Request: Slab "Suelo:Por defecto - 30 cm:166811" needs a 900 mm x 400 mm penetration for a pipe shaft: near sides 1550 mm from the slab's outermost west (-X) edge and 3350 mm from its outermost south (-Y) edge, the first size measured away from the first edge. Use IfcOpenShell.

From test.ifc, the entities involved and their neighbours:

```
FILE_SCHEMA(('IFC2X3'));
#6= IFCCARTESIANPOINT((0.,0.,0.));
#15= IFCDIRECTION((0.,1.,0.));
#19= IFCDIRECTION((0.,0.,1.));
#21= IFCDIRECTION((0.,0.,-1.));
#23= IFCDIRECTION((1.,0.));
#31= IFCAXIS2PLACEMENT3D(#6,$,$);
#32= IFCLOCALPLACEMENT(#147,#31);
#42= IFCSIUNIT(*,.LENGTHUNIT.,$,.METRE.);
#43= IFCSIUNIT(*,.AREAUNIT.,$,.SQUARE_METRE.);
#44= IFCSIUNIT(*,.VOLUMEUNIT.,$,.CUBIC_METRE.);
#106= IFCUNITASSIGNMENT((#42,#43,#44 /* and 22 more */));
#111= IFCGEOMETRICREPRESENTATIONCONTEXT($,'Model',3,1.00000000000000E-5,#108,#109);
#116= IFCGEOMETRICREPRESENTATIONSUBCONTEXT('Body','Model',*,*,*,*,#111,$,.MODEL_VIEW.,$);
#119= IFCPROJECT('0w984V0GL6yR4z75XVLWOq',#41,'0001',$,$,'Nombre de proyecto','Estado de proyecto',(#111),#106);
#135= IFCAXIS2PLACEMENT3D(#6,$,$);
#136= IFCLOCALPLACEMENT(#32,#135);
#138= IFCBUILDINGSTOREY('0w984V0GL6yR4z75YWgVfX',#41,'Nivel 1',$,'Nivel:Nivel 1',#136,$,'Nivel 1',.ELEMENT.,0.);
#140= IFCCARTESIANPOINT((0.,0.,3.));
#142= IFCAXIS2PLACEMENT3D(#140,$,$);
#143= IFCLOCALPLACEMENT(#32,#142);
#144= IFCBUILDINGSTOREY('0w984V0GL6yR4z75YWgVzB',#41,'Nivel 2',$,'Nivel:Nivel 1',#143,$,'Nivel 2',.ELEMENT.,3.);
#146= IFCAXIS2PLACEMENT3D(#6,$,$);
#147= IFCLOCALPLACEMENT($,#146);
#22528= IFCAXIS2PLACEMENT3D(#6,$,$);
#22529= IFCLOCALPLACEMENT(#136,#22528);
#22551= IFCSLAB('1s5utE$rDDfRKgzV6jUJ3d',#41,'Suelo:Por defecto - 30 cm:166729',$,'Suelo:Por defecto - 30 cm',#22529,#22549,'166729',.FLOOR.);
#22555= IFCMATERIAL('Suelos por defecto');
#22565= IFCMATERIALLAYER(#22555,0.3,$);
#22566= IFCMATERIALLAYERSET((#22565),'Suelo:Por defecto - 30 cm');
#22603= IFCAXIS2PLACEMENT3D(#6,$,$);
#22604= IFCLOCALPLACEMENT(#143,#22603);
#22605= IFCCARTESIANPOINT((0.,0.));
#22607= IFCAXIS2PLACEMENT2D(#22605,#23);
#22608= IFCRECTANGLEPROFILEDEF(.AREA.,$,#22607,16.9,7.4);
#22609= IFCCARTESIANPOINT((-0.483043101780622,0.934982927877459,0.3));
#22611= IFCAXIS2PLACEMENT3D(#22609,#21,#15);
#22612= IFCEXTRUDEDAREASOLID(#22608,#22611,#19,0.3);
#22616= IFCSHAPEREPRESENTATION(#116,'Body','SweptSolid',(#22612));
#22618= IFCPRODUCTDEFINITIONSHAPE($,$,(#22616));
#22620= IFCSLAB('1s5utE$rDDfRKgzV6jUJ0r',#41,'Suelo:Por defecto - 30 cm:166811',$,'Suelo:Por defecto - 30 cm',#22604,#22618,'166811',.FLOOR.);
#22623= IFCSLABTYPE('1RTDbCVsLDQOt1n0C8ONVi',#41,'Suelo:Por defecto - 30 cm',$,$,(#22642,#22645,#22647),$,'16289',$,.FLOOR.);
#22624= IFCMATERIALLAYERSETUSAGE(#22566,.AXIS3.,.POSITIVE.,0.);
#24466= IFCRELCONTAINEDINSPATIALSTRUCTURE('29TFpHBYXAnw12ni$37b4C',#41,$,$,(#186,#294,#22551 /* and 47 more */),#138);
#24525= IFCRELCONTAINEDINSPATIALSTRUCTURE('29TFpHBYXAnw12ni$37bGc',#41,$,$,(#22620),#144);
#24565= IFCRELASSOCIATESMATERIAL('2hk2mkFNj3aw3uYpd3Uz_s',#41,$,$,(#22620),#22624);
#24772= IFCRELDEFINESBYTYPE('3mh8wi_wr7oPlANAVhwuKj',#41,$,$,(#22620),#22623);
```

```python
import numpy as np
import ifcopenshell
import ifcopenshell.api.feature
import ifcopenshell.api.geometry
import ifcopenshell.api.root
import ifcopenshell.geom
import ifcopenshell.util.placement
import ifcopenshell.util.representation
import ifcopenshell.util.shape
import ifcopenshell.util.unit

model = ifcopenshell.open("test.ifc")
unit_scale = ifcopenshell.util.unit.calculate_unit_scale(model)
settings = ifcopenshell.geom.settings()


def volume(element):
    """Net volume in cubic metres, openings subtracted."""
    shape = ifcopenshell.geom.create_shape(settings, element)
    return ifcopenshell.util.shape.get_volume(shape.geometry)


slab = model.by_guid("1s5utE$rDDfRKgzV6jUJ0r")
before = volume(slab)

# Extent in the slab's own axes, in metres. The edges named are its -X and -Y sides.
slab_shape = ifcopenshell.geom.create_shape(settings, slab)
vertices = ifcopenshell.util.shape.get_vertices(slab_shape.geometry)
x_min, y_min, bottom = vertices.min(axis=0)
top = vertices[:, 2].max()

opening = ifcopenshell.api.root.create_entity(model, ifc_class="IfcOpeningElement", name="Pipe shaft opening")
context = ifcopenshell.util.representation.get_context(model, "Model", "Body", "MODEL_VIEW")
width, depth = 0.9, 0.4
outline = [(0.0, 0.0), (width, 0.0), (width, depth), (0.0, depth), (0.0, 0.0)]
# Overshoot both faces by 50 mm so the cut is clean.
shape = ifcopenshell.api.geometry.add_slab_representation(
    model, context=context, depth=top - bottom + 0.1, polyline=outline
)
ifcopenshell.api.geometry.assign_representation(model, product=opening, representation=shape)

matrix = ifcopenshell.util.placement.get_local_placement(slab.ObjectPlacement)
matrix[:, 3] = matrix @ np.append(np.array([x_min + 1.55, y_min + 3.35, bottom - 0.05]) / unit_scale, 1.0)
ifcopenshell.api.geometry.edit_object_placement(model, product=opening, matrix=matrix, is_si=False)
ifcopenshell.api.feature.add_feature(model, feature=opening, element=slab)

after = volume(slab)

print(f"slab volume {before:.3f} -> {after:.3f} m3")

model.write("test_edited.ifc")
```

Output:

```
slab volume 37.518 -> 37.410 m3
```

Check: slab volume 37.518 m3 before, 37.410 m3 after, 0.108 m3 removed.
